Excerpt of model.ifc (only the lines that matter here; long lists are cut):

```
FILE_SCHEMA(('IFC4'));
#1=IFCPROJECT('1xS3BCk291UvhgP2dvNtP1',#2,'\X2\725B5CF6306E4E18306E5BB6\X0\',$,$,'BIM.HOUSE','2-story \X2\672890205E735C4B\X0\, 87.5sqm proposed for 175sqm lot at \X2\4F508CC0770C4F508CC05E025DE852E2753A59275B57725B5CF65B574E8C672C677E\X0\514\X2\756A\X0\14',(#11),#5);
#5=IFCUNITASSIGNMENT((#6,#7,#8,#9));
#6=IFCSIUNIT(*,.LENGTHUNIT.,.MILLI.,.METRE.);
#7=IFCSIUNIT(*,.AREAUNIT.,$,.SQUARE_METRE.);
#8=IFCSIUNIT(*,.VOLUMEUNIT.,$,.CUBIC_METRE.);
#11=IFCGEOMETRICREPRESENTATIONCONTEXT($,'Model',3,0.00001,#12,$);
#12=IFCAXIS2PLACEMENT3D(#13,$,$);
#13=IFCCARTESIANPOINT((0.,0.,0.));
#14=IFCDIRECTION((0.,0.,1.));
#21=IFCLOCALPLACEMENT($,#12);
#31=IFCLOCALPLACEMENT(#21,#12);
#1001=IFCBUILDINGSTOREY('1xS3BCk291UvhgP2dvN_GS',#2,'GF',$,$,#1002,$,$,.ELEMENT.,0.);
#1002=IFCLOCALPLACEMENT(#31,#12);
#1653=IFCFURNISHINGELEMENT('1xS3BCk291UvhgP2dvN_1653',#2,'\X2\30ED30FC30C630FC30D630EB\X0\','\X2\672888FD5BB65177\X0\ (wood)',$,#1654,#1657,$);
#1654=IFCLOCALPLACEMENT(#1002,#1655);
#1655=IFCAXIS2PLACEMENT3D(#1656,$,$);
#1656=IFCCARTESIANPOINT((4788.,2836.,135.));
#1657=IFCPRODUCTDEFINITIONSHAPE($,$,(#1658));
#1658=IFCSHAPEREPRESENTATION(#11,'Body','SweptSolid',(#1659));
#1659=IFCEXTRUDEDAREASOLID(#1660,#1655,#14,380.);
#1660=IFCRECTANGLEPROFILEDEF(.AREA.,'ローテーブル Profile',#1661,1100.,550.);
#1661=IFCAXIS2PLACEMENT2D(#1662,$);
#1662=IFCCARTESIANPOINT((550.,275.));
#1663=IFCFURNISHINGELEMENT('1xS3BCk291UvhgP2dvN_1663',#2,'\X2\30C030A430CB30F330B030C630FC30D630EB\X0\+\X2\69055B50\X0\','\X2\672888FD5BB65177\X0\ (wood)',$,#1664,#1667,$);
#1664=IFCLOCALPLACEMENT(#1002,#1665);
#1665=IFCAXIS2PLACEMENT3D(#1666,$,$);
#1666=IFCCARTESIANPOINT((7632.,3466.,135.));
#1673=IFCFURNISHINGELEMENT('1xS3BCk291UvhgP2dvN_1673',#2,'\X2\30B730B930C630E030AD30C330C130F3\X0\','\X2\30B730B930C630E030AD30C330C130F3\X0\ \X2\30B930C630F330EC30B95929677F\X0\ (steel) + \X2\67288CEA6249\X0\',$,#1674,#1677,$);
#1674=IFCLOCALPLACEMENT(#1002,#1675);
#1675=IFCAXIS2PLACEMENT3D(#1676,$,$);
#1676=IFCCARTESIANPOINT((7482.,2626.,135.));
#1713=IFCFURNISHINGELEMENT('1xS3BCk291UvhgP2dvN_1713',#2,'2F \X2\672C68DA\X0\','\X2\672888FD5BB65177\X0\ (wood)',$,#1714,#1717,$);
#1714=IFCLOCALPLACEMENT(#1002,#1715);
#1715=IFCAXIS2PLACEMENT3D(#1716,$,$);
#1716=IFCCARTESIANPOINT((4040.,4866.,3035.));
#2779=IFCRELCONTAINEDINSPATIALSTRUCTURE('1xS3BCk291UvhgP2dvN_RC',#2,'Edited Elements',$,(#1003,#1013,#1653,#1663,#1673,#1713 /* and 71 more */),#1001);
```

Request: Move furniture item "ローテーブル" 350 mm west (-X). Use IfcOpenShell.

```python
import ifcopenshell
import ifcopenshell.api.geometry
import ifcopenshell.util.placement
import ifcopenshell.util.unit

model = ifcopenshell.open("model.ifc")
unit_scale = ifcopenshell.util.unit.calculate_unit_scale(model)

item = model.by_id(1653)
matrix = ifcopenshell.util.placement.get_local_placement(item.ObjectPlacement)
matrix[0, 3] -= 0.35 / unit_scale
ifcopenshell.api.geometry.edit_object_placement(model, product=item, matrix=matrix, is_si=False)

print(ifcopenshell.util.placement.get_local_placement(item.ObjectPlacement).round(3) + 0.0)

model.write("model_edited.ifc")
```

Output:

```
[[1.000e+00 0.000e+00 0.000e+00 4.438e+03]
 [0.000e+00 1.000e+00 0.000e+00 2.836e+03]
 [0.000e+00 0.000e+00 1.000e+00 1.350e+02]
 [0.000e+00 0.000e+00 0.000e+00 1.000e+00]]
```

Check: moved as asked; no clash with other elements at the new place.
